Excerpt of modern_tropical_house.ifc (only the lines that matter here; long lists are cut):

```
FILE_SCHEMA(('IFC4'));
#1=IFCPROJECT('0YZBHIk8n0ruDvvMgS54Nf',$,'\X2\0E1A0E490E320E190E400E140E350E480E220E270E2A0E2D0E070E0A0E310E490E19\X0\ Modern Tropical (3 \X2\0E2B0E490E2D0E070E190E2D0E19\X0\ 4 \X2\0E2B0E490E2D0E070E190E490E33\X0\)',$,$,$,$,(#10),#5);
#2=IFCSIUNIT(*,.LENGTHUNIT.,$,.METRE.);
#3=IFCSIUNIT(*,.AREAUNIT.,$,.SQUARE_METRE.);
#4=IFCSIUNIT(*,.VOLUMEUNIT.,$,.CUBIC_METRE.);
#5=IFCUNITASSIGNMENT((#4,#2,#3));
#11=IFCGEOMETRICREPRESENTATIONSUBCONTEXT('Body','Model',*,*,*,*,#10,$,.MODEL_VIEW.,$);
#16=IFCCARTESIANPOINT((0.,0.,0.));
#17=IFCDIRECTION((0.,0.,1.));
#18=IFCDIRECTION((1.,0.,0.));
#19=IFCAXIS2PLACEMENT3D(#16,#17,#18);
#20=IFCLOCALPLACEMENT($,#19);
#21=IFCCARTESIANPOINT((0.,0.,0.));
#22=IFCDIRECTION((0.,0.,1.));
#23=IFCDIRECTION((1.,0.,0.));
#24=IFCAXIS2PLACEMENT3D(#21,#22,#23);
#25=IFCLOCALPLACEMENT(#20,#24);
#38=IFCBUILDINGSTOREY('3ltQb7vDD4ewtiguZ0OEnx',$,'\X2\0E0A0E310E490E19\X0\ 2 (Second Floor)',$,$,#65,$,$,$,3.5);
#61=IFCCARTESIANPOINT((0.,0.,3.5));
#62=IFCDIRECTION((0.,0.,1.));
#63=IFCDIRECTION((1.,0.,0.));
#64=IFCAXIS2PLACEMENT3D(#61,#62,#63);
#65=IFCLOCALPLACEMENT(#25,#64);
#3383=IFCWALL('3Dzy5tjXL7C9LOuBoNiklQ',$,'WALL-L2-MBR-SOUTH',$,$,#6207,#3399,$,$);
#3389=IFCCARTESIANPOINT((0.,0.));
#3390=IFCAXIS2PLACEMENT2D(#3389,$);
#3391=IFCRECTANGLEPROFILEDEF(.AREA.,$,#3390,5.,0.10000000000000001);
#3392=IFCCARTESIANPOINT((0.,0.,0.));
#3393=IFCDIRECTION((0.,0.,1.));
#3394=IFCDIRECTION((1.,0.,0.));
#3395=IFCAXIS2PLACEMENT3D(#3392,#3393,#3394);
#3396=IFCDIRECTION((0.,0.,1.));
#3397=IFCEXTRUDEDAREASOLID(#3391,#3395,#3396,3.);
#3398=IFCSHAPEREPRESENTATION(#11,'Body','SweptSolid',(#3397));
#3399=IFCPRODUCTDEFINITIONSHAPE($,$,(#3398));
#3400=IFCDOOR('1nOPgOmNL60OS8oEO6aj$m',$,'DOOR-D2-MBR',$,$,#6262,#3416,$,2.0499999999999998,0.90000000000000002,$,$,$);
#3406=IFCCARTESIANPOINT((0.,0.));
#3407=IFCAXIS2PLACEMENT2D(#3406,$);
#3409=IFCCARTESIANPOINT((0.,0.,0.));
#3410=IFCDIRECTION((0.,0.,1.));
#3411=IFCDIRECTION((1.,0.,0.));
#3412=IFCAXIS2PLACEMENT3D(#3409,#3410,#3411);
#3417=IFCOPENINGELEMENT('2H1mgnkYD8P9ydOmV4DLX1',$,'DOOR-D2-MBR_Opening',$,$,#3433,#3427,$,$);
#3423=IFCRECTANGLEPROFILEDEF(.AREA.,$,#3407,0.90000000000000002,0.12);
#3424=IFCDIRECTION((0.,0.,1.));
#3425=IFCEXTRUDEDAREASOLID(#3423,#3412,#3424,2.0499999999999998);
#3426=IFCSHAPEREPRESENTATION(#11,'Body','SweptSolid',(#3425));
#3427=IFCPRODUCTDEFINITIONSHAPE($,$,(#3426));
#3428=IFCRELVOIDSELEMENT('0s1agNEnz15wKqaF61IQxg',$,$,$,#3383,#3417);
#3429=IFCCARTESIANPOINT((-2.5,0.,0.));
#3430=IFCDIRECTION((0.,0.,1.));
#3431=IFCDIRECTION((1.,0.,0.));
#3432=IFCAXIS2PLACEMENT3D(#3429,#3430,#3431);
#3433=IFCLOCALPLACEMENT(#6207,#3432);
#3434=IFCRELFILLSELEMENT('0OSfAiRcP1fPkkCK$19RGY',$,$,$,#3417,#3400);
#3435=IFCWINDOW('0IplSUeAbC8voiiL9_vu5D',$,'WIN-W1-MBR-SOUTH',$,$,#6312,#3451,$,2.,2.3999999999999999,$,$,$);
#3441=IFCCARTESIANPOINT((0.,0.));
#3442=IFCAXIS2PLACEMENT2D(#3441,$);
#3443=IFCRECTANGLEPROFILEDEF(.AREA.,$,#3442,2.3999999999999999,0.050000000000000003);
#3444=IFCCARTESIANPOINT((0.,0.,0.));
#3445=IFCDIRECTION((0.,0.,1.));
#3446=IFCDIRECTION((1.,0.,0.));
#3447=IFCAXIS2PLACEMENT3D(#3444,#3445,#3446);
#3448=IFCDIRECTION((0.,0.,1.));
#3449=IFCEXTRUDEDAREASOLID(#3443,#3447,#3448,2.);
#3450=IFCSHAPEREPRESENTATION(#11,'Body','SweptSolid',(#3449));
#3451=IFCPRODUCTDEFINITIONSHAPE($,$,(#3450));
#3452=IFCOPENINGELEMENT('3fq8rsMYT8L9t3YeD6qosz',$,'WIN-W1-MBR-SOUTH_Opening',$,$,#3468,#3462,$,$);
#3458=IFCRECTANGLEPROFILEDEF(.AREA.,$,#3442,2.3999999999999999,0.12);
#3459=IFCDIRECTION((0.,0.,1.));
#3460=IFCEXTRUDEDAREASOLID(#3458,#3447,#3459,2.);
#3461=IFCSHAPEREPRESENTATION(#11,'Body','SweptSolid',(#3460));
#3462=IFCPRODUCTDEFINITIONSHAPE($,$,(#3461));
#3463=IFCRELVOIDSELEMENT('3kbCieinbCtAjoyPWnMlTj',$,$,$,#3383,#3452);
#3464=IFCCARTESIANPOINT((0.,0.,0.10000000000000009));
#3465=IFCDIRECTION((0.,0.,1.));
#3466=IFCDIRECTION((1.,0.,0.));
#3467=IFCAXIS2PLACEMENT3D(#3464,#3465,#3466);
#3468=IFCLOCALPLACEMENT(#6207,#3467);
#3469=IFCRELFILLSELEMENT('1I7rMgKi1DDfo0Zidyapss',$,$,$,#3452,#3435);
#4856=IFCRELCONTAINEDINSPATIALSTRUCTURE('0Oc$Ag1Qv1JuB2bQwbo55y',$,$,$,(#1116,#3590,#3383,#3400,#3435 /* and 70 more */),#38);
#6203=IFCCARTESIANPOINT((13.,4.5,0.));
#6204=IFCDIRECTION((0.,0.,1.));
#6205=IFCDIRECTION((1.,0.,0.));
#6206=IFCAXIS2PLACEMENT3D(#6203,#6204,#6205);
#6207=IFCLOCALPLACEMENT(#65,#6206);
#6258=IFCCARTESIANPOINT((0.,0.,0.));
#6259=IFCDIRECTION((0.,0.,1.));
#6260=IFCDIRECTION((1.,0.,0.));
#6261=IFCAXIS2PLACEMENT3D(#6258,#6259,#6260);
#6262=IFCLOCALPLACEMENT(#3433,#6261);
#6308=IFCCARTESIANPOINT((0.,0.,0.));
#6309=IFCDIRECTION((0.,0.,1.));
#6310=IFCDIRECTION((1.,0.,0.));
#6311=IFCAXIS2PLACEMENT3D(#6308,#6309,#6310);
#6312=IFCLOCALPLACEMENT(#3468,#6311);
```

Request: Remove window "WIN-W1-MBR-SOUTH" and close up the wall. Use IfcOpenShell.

```python
import ifcopenshell
import ifcopenshell.api.feature
import ifcopenshell.api.root
import ifcopenshell.geom
import ifcopenshell.util.shape

model = ifcopenshell.open("modern_tropical_house.ifc")
settings = ifcopenshell.geom.settings()


def volume(element):
    """Net volume in cubic metres, openings subtracted."""
    shape = ifcopenshell.geom.create_shape(settings, element)
    return ifcopenshell.util.shape.get_volume(shape.geometry)


window = model.by_guid("0IplSUeAbC8voiiL9_vu5D")
opening = window.FillsVoids[0].RelatingOpeningElement
wall = opening.VoidsElements[0].RelatingBuildingElement
before = volume(wall)

ifcopenshell.api.root.remove_product(model, product=window)
ifcopenshell.api.feature.remove_feature(model, feature=opening)

after = volume(wall)

print(f"wall volume {before:.3f} -> {after:.3f} m3")

model.write("modern_tropical_house_updated.ifc")
```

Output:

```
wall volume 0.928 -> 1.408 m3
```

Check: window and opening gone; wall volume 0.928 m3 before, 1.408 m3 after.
